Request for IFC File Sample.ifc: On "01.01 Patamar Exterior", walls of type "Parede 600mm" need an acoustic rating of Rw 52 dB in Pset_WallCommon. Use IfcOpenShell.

First a look at what the model holds.

```python
import ifcopenshell
import ifcopenshell.util.element

model = ifcopenshell.open("IFC File Sample.ifc")
print(model.schema)
storey = next(s for s in model.by_type("IfcBuildingStorey") if s.Name == "01.01 Patamar Exterior")
walls = [e for e in ifcopenshell.util.element.get_decomposition(storey) if e.is_a("IfcWall")]
seen = {}
for e in walls:
    element_type = ifcopenshell.util.element.get_type(e)
    key = (element_type.Name if element_type != e and element_type else None, ifcopenshell.util.element.get_pset(e, "Pset_WallCommon", "AcousticRating"))
    seen[key] = seen.get(key, 0) + 1
for (name, value), count in sorted(seen.items(), key=str):
    print(count, "x", name, "|", value)
```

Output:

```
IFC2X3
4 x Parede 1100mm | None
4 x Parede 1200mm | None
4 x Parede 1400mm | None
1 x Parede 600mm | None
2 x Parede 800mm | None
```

```python
import ifcopenshell
import ifcopenshell.api.pset
import ifcopenshell.util.element

model = ifcopenshell.open("IFC File Sample.ifc")

storey = next(s for s in model.by_type("IfcBuildingStorey") if s.Name == "01.01 Patamar Exterior")
walls = [e for e in ifcopenshell.util.element.get_decomposition(storey) if e.is_a("IfcWall")]

count = 0
for e in walls:
    element_type = ifcopenshell.util.element.get_type(e)
    if element_type in (None, e) or element_type.Name != "Parede 600mm":
        continue
    # add_pset returns the element's existing set when there is one.
    pset = ifcopenshell.api.pset.add_pset(model, product=e, name="Pset_WallCommon")
    ifcopenshell.api.pset.edit_pset(model, pset=pset, properties={"AcousticRating": "Rw 52 dB"})
    count += 1

print(count, "walls updated")

model.write("IFC File Sample_edited.ifc")
```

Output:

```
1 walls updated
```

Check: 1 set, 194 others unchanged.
